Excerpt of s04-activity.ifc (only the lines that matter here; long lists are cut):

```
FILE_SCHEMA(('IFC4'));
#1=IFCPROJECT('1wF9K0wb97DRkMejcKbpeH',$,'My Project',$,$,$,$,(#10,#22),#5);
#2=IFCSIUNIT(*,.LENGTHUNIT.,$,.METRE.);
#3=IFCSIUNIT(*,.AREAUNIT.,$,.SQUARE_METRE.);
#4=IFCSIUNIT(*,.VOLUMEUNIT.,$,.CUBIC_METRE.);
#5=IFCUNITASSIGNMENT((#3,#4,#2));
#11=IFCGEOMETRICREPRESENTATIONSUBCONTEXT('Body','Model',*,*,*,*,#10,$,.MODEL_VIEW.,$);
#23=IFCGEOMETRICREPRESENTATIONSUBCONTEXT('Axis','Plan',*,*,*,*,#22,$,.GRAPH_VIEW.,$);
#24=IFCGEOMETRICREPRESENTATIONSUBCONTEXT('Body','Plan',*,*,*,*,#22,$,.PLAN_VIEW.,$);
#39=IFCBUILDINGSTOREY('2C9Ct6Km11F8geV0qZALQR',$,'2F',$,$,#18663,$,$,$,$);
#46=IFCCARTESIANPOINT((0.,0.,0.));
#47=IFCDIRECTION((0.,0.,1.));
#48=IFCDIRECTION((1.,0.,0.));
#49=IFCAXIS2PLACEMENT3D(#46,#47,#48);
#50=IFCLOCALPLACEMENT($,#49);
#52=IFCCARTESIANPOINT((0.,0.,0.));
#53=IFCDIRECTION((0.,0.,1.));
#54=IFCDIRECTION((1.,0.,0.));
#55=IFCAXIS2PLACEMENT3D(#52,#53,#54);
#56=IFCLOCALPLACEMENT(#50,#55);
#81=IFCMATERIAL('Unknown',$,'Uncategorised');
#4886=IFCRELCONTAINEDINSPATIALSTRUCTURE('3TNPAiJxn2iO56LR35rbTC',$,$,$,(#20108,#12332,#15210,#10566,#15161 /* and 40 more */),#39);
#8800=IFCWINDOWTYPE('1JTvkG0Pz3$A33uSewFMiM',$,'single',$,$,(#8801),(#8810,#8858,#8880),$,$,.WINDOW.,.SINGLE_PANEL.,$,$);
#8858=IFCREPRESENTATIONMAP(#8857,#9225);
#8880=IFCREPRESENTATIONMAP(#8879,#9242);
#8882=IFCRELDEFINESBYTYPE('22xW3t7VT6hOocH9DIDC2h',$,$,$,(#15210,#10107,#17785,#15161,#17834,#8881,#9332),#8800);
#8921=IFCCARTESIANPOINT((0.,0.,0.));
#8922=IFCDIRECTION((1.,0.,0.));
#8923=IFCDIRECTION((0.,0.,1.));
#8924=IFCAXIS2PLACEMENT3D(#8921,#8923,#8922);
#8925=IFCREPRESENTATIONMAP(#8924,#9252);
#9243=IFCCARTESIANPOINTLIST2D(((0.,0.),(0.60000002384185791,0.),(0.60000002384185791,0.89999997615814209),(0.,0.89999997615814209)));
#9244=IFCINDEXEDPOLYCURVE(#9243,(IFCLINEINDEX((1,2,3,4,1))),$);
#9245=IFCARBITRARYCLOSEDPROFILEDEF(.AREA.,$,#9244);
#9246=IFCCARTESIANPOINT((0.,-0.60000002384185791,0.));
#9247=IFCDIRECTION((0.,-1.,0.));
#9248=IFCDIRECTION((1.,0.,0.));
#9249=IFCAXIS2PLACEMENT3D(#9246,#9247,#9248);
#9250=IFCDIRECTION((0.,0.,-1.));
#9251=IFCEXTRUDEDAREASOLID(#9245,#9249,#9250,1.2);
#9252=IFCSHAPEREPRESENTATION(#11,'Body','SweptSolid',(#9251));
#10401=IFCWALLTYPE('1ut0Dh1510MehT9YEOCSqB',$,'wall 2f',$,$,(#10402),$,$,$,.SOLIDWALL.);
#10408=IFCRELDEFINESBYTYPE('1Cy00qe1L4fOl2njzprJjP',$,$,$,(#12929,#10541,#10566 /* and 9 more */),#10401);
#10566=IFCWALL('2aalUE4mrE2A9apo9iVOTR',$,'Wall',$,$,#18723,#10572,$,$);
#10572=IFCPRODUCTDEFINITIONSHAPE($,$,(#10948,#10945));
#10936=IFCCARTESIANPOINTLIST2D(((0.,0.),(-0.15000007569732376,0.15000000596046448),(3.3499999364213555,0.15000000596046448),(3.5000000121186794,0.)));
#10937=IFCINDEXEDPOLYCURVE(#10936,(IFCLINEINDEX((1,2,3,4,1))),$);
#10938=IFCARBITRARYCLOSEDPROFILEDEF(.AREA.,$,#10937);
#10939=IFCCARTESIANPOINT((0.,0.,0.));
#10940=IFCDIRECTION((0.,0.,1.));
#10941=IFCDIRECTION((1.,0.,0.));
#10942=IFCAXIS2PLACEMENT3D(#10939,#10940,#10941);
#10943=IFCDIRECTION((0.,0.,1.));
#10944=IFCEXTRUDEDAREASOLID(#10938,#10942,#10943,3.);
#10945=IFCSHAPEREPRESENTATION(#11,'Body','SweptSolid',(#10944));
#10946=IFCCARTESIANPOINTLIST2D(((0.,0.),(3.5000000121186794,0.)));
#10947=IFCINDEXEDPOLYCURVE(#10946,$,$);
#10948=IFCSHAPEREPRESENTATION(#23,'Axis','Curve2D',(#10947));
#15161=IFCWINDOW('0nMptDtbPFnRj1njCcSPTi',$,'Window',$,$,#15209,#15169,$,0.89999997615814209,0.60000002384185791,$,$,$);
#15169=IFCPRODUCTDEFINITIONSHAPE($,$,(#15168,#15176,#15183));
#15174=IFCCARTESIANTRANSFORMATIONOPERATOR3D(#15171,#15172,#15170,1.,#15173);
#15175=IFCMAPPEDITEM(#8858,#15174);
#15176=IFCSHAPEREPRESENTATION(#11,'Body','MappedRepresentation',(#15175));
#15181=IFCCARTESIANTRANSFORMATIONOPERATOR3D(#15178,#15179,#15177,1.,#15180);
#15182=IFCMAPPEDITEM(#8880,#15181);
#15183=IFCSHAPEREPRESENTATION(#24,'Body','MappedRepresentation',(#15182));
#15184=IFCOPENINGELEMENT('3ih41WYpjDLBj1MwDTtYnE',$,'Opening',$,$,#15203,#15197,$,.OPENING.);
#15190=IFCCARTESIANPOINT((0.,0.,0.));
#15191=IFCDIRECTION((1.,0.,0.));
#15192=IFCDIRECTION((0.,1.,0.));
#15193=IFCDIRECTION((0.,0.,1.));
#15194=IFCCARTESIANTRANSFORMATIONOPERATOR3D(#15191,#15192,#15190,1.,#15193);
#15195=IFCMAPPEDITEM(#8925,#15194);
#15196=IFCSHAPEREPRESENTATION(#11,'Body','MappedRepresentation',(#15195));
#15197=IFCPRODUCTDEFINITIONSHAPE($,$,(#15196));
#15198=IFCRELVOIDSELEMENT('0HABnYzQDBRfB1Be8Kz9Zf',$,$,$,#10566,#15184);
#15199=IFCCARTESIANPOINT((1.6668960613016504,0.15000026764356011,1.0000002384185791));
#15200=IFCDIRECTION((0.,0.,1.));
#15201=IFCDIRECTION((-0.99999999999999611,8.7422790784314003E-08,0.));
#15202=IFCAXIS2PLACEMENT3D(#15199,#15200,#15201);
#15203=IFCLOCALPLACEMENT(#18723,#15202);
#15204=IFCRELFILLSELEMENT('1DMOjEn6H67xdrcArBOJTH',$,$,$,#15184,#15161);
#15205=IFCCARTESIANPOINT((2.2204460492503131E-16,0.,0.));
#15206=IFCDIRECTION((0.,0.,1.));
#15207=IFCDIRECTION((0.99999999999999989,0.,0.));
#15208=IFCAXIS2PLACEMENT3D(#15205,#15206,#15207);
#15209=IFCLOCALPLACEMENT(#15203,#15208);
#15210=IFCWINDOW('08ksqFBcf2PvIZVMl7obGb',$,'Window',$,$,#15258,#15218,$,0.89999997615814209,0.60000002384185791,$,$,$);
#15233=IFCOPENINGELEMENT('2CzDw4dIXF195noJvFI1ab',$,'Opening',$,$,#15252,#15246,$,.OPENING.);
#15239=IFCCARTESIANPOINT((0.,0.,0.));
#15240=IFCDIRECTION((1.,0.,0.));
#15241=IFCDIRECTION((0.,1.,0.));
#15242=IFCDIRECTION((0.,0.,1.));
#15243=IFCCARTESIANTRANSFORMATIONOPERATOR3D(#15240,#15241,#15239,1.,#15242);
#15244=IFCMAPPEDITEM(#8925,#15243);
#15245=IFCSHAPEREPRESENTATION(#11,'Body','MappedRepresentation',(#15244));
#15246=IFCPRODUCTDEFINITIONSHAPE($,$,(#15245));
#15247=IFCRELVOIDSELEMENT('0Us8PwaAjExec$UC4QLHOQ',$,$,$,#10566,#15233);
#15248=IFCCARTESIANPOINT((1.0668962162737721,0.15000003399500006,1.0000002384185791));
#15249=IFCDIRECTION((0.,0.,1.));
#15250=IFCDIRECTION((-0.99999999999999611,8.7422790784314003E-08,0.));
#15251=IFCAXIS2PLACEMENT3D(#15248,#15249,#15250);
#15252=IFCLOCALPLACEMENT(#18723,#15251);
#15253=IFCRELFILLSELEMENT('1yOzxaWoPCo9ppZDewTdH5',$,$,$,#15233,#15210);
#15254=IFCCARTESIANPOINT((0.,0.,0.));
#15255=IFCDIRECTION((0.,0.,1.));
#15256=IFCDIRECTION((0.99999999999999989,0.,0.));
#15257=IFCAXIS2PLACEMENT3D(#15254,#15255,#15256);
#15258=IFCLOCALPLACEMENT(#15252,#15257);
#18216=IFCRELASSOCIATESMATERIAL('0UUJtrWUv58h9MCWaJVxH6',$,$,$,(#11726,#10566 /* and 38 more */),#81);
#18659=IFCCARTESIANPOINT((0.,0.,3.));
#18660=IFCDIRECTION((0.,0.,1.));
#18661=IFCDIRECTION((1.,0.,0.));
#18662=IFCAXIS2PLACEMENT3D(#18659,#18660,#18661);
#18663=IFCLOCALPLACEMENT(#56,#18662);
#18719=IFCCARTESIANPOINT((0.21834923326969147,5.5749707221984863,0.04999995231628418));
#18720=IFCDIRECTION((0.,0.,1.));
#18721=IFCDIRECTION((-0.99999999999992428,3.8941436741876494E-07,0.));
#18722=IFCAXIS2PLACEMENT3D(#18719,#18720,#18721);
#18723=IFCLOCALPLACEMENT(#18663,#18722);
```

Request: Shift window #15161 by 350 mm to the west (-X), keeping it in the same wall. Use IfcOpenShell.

```python
import ifcopenshell
import ifcopenshell.api.geometry
import ifcopenshell.util.placement
import ifcopenshell.util.unit

model = ifcopenshell.open("s04-activity.ifc")
unit_scale = ifcopenshell.util.unit.calculate_unit_scale(model)

window = model.by_guid("0nMptDtbPFnRj1njCcSPTi")
opening = window.FillsVoids[0].RelatingOpeningElement
wall = opening.VoidsElements[0].RelatingBuildingElement

wall_matrix = ifcopenshell.util.placement.get_local_placement(wall.ObjectPlacement)
shift = wall_matrix[:3, 0] * 0.35 / unit_scale
before = ifcopenshell.util.placement.get_local_placement(window.ObjectPlacement)[:3, 3].copy()

# The window is placed relative to its opening, so it follows when the opening moves.
matrix = ifcopenshell.util.placement.get_local_placement(opening.ObjectPlacement)
matrix[:3, 3] += shift
ifcopenshell.api.geometry.edit_object_placement(
    model, product=opening, matrix=matrix, is_si=False, should_transform_children=True
)

after = ifcopenshell.util.placement.get_local_placement(window.ObjectPlacement)[:3, 3]
print("window moved by", (after - before).round(3) + 0.0)

model.write("s04-activity_updated.ifc")
```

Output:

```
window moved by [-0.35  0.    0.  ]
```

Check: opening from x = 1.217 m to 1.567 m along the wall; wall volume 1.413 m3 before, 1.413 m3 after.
